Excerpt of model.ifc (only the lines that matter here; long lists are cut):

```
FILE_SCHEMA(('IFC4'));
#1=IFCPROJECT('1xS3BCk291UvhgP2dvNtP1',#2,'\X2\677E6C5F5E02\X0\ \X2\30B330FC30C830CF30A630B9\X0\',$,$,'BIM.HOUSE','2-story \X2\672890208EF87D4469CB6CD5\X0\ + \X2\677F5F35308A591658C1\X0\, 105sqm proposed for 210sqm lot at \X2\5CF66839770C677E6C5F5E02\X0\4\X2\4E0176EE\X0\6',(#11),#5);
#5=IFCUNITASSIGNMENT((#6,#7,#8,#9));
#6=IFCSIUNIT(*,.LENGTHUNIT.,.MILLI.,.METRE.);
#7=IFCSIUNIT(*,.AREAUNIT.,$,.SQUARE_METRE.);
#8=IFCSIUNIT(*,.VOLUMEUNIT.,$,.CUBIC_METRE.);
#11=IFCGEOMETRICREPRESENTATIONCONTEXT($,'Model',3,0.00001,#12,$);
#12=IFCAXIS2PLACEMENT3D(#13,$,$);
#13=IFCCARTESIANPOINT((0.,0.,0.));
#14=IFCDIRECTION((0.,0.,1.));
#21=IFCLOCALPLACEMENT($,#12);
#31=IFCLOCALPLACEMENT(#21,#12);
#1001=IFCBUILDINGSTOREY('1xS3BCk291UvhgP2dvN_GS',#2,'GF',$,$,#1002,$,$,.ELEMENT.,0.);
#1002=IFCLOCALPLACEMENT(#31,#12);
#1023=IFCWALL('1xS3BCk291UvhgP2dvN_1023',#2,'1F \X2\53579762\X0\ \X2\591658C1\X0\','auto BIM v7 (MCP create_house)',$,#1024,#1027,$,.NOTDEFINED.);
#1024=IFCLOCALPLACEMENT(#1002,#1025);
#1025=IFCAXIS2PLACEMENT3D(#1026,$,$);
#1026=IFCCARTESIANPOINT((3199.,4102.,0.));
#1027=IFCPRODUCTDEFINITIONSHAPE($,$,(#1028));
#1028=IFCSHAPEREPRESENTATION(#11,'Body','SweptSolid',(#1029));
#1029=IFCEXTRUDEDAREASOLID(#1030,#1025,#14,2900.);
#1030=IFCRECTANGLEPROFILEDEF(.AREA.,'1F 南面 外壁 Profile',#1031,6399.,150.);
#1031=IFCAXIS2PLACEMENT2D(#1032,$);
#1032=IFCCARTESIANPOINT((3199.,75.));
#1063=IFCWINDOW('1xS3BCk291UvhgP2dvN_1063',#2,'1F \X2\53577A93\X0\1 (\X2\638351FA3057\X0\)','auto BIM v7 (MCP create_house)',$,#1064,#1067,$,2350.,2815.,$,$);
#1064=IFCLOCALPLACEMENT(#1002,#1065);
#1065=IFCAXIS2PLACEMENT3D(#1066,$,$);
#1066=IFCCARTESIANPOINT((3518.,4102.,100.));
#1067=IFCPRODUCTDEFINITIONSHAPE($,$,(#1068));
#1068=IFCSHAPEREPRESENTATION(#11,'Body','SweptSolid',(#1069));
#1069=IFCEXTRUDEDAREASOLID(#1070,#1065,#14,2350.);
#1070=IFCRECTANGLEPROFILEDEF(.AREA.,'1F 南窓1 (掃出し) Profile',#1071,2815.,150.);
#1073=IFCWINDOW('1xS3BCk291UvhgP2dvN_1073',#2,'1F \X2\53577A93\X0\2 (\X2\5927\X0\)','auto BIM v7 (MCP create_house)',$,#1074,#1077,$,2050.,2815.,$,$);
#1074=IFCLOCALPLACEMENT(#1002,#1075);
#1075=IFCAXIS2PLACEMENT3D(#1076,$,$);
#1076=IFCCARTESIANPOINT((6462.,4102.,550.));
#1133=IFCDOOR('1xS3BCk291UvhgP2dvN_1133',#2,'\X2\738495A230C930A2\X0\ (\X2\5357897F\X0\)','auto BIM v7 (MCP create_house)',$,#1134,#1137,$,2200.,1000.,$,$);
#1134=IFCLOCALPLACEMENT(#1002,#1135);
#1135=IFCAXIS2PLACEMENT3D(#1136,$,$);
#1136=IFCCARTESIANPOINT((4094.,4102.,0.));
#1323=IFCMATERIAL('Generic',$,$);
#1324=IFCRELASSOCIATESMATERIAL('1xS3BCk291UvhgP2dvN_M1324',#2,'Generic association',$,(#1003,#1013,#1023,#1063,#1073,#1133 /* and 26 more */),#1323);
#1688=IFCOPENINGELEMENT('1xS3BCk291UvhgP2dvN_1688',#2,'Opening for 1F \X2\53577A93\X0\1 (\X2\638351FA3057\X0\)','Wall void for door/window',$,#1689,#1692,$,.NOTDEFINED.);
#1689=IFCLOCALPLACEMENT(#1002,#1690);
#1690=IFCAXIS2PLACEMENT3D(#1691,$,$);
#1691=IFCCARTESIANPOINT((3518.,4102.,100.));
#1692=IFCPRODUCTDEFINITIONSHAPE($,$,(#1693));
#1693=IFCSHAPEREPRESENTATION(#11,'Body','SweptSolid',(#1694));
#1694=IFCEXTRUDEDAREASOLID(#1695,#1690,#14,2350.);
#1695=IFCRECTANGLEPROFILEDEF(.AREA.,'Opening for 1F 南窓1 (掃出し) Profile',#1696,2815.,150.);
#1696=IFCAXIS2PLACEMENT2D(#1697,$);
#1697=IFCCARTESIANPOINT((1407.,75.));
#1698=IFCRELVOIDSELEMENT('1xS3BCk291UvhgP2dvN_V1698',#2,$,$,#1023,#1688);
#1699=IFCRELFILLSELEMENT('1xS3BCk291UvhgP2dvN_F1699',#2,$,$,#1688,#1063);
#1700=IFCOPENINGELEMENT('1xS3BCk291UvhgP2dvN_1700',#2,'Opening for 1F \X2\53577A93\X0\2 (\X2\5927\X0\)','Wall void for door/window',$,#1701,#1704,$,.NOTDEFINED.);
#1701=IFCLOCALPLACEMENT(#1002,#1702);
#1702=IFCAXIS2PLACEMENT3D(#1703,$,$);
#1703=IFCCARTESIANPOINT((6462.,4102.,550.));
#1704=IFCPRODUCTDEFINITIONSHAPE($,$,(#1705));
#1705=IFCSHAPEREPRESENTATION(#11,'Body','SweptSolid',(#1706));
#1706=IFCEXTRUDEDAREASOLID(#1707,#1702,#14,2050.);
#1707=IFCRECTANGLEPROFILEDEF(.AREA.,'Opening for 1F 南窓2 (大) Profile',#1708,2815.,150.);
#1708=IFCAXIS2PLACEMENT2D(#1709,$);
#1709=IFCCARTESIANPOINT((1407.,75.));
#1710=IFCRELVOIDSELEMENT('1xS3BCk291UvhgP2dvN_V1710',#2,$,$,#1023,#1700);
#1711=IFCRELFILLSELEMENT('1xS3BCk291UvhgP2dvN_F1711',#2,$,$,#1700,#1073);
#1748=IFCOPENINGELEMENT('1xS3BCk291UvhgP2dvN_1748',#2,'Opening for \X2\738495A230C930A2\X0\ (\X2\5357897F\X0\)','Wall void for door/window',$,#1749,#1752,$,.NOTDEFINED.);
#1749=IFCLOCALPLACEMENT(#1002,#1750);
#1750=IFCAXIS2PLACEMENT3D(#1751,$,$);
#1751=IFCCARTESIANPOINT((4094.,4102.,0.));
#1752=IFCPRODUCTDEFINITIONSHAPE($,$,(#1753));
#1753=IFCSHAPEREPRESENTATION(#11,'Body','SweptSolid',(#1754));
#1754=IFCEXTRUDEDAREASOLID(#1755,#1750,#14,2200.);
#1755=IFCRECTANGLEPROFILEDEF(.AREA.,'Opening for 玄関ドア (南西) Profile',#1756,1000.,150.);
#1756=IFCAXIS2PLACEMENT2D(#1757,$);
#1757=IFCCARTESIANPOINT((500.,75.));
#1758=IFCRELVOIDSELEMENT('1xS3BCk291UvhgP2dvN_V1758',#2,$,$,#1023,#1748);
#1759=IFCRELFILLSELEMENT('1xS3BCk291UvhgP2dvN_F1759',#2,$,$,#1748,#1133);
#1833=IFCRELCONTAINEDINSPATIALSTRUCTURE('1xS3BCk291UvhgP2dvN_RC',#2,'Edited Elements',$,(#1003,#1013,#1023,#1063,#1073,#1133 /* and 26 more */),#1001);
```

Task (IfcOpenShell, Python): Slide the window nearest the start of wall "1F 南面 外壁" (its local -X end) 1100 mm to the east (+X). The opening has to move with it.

```python
import ifcopenshell
import ifcopenshell.api.geometry
import ifcopenshell.util.placement
import ifcopenshell.util.unit

model = ifcopenshell.open("model.ifc")
unit_scale = ifcopenshell.util.unit.calculate_unit_scale(model)

window = model.by_guid("1xS3BCk291UvhgP2dvN_1063")
opening = window.FillsVoids[0].RelatingOpeningElement
wall = opening.VoidsElements[0].RelatingBuildingElement

wall_matrix = ifcopenshell.util.placement.get_local_placement(wall.ObjectPlacement)
shift = wall_matrix[:3, 0] * 1.1 / unit_scale
before = ifcopenshell.util.placement.get_local_placement(window.ObjectPlacement)[:3, 3].copy()

# The window is not placed relative to its opening, so move both.
for product in (opening, window):
    matrix = ifcopenshell.util.placement.get_local_placement(product.ObjectPlacement)
    matrix[:3, 3] += shift
    ifcopenshell.api.geometry.edit_object_placement(model, product=product, matrix=matrix, is_si=False)

after = ifcopenshell.util.placement.get_local_placement(window.ObjectPlacement)[:3, 3]
print("window moved by", (after - before).round(3) + 0.0)

model.write("model-out.ifc")
```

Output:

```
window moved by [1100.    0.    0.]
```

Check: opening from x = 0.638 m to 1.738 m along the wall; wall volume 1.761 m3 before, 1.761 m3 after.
